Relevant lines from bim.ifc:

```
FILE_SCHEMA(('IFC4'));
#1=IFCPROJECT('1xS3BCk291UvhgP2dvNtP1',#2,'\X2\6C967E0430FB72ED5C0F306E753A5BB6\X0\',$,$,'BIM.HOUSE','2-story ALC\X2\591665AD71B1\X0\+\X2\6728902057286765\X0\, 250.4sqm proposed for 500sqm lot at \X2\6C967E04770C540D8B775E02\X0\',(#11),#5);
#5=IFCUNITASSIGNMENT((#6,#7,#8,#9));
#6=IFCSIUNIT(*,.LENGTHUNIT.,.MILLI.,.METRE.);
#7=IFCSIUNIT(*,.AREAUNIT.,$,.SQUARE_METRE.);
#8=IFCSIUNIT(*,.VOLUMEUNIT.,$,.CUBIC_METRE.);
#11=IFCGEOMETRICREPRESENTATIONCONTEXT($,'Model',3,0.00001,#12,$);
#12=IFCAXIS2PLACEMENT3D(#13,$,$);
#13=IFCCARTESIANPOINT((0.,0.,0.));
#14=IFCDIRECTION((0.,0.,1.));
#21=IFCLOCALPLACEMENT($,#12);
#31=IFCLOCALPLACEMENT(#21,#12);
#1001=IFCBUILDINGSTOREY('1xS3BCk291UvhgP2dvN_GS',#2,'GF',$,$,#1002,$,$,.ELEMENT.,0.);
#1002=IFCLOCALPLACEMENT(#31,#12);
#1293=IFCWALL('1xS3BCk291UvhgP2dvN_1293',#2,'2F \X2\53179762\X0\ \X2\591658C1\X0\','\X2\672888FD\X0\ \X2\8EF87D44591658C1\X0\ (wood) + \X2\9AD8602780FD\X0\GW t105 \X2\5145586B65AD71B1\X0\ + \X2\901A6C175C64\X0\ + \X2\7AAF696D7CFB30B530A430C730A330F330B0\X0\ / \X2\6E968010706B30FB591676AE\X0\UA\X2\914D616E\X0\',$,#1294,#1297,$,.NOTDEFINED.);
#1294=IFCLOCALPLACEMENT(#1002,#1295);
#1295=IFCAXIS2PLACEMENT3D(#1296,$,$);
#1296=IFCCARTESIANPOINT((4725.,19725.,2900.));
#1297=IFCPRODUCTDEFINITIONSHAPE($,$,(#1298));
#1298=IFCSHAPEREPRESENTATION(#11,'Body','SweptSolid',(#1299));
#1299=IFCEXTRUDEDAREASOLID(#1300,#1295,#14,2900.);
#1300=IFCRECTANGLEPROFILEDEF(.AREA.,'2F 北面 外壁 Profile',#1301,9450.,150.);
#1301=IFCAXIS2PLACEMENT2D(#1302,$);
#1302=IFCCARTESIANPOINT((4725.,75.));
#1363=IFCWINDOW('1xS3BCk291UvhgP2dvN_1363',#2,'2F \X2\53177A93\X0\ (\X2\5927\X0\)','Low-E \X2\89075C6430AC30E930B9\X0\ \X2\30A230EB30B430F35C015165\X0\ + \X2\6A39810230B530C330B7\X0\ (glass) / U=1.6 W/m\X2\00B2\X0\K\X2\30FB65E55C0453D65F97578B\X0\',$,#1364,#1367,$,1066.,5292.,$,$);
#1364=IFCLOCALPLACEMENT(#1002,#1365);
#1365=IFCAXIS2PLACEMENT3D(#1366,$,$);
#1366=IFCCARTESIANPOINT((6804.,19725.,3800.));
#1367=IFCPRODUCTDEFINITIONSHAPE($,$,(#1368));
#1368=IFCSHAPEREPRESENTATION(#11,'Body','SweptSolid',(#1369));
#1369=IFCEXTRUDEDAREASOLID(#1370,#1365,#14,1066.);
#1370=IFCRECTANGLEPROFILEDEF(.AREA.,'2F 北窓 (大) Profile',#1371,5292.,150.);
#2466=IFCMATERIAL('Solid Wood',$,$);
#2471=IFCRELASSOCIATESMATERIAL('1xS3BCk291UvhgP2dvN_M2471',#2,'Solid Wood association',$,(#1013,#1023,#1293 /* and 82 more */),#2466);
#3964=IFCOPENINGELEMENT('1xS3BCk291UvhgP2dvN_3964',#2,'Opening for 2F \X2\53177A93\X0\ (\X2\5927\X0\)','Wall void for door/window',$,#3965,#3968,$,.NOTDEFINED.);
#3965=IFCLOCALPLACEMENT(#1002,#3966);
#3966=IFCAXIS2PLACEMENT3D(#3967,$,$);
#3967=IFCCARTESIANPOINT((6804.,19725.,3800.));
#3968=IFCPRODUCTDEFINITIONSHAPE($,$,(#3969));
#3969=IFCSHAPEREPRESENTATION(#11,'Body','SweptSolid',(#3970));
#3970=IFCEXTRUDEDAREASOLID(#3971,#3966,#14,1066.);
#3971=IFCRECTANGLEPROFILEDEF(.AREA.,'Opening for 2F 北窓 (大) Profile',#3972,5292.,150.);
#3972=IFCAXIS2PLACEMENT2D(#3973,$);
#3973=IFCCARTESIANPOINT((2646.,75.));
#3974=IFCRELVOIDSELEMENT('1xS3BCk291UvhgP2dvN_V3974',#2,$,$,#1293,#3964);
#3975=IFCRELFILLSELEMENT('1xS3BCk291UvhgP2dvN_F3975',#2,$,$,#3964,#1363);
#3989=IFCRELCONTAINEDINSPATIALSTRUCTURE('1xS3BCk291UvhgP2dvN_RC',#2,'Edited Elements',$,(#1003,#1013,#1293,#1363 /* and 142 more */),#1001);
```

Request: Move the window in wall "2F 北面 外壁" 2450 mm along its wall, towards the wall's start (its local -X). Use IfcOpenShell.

```python
import ifcopenshell
import ifcopenshell.api.geometry
import ifcopenshell.util.placement
import ifcopenshell.util.unit

model = ifcopenshell.open("bim.ifc")
unit_scale = ifcopenshell.util.unit.calculate_unit_scale(model)

window = model.by_id(1363)
opening = window.FillsVoids[0].RelatingOpeningElement
wall = opening.VoidsElements[0].RelatingBuildingElement

wall_matrix = ifcopenshell.util.placement.get_local_placement(wall.ObjectPlacement)
shift = wall_matrix[:3, 0] * -2.45 / unit_scale
before = ifcopenshell.util.placement.get_local_placement(window.ObjectPlacement)[:3, 3].copy()

# The window is not placed relative to its opening, so move both.
for product in (opening, window):
    matrix = ifcopenshell.util.placement.get_local_placement(product.ObjectPlacement)
    matrix[:3, 3] += shift
    ifcopenshell.api.geometry.edit_object_placement(model, product=product, matrix=matrix, is_si=False)

after = ifcopenshell.util.placement.get_local_placement(window.ObjectPlacement)[:3, 3]
print("window moved by", (after - before).round(3) + 0.0)

model.write("bim-out.ifc")
```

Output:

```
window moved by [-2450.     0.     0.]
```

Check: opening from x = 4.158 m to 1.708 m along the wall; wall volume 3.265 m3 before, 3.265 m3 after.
